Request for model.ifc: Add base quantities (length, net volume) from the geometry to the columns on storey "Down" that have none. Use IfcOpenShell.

First a look at what the model holds.

```python
import ifcopenshell
import ifcopenshell.util.element
import ifcopenshell.util.unit

model = ifcopenshell.open("model.ifc")
print(model.schema)
for unit_type in ("LENGTHUNIT", "AREAUNIT", "VOLUMEUNIT"):
    print(unit_type, ifcopenshell.util.unit.calculate_unit_scale(model, unit_type))
storey = next(s for s in model.by_type("IfcBuildingStorey") if s.Name == "Down")
columns = [e for e in ifcopenshell.util.element.get_decomposition(storey) if e.is_a("IfcColumn")]
for e in sorted(columns, key=lambda e: e.id()):
    print(e.id(), e.is_a(), e.Name, list(ifcopenshell.util.element.get_psets(e, qtos_only=True)), sep=" | ")
```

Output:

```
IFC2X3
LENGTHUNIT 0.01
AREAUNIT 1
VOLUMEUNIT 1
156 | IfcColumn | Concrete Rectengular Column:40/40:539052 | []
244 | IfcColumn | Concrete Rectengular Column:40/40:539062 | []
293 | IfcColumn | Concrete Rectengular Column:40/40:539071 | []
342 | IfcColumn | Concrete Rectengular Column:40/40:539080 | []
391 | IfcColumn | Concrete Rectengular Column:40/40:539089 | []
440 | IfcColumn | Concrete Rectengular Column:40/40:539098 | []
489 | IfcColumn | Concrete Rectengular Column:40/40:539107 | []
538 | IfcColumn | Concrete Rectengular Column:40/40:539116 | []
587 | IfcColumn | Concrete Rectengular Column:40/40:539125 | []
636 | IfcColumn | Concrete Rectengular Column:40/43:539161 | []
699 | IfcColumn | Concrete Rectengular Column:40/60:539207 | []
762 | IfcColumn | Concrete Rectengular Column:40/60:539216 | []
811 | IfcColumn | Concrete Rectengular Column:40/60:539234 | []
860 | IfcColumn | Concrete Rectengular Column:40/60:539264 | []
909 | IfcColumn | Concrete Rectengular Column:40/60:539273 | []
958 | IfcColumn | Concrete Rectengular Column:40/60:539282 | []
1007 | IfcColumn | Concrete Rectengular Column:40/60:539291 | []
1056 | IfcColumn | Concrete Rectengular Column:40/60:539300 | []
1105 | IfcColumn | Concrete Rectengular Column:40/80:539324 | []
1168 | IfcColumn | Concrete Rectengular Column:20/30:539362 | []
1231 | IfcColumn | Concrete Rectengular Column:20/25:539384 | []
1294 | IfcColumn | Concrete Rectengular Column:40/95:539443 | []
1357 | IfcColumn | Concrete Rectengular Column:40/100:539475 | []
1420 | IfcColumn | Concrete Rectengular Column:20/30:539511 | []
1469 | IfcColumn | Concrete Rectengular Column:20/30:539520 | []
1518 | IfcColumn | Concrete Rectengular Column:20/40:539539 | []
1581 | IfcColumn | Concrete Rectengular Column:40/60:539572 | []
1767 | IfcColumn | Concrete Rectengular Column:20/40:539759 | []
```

```python
import ifcopenshell
import ifcopenshell.api.pset
import ifcopenshell.geom
import ifcopenshell.util.element
import ifcopenshell.util.shape
import ifcopenshell.util.unit

model = ifcopenshell.open("model.ifc")
unit_scale = ifcopenshell.util.unit.calculate_unit_scale(model)
volume_scale = ifcopenshell.util.unit.calculate_unit_scale(model, "VOLUMEUNIT")
settings = ifcopenshell.geom.settings()

storey = next(s for s in model.by_type("IfcBuildingStorey") if s.Name == "Down")
columns = [e for e in ifcopenshell.util.element.get_decomposition(storey) if e.is_a("IfcColumn")]

for e in sorted(columns, key=lambda e: e.id()):
    if ifcopenshell.util.element.get_psets(e, qtos_only=True, should_inherit=False):
        continue
    # Geometry comes back in metres, in the element's own axes.
    shape = ifcopenshell.geom.create_shape(settings, e)
    values = {
        "Length": ifcopenshell.util.shape.get_z(shape.geometry) / unit_scale,
        "NetVolume": ifcopenshell.util.shape.get_volume(shape.geometry) / volume_scale,
    }
    qto = ifcopenshell.api.pset.add_qto(model, product=e, name="BaseQuantities")
    ifcopenshell.api.pset.edit_qto(model, qto=qto, properties=values)
    print(e.id(), {k: round(v, 3) for k, v in values.items()})

model.write("model_edited.ifc")
```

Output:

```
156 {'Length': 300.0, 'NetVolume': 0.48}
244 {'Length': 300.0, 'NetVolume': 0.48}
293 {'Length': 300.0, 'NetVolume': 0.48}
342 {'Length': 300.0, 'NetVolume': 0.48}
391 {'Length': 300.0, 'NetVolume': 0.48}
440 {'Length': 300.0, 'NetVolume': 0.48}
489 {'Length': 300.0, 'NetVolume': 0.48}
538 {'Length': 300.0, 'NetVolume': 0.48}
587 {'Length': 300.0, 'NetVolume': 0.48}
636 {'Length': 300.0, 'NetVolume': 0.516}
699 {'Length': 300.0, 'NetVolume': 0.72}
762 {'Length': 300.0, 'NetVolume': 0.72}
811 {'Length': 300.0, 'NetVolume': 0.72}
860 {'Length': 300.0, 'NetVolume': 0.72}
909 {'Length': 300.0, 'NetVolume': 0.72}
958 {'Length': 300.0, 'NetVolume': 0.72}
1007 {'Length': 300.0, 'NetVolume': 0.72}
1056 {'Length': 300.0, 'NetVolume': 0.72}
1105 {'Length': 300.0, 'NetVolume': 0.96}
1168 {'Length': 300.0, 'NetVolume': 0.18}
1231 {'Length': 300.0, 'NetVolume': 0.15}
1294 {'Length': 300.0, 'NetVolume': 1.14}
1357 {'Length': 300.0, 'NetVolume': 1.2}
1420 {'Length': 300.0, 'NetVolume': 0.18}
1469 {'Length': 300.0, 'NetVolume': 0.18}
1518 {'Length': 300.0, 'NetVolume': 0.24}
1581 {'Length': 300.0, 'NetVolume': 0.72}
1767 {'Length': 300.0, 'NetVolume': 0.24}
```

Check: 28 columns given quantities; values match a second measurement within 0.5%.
